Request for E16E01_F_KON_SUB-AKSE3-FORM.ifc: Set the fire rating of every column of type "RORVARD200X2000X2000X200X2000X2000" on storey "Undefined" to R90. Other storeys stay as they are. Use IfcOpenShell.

First a look at what the model holds.

```python
import ifcopenshell
import ifcopenshell.util.element

model = ifcopenshell.open("E16E01_F_KON_SUB-AKSE3-FORM.ifc")
print(model.schema)
storey = next(s for s in model.by_type("IfcBuildingStorey") if s.Name == "Undefined")
columns = [e for e in ifcopenshell.util.element.get_decomposition(storey) if e.is_a("IfcColumn")]
seen = {}
for e in columns:
    element_type = ifcopenshell.util.element.get_type(e)
    key = (element_type.Name if element_type != e and element_type else None, ifcopenshell.util.element.get_pset(e, "Pset_ColumnCommon", "FireRating"))
    seen[key] = seen.get(key, 0) + 1
for (name, value), count in sorted(seen.items(), key=str):
    print(count, "x", name, "|", value)
```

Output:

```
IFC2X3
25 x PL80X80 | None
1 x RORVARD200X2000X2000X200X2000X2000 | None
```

```python
import ifcopenshell
import ifcopenshell.api.pset
import ifcopenshell.util.element

model = ifcopenshell.open("E16E01_F_KON_SUB-AKSE3-FORM.ifc")

storey = next(s for s in model.by_type("IfcBuildingStorey") if s.Name == "Undefined")
columns = [e for e in ifcopenshell.util.element.get_decomposition(storey) if e.is_a("IfcColumn")]

count = 0
for e in columns:
    element_type = ifcopenshell.util.element.get_type(e)
    if element_type in (None, e) or element_type.Name != "RORVARD200X2000X2000X200X2000X2000":
        continue
    # add_pset returns the element's existing set when there is one.
    pset = ifcopenshell.api.pset.add_pset(model, product=e, name="Pset_ColumnCommon")
    ifcopenshell.api.pset.edit_pset(model, pset=pset, properties={"FireRating": "R90"})
    count += 1

print(count, "columns updated")

model.write("E16E01_F_KON_SUB-AKSE3-FORM-out.ifc")
```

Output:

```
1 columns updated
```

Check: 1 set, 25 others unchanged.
